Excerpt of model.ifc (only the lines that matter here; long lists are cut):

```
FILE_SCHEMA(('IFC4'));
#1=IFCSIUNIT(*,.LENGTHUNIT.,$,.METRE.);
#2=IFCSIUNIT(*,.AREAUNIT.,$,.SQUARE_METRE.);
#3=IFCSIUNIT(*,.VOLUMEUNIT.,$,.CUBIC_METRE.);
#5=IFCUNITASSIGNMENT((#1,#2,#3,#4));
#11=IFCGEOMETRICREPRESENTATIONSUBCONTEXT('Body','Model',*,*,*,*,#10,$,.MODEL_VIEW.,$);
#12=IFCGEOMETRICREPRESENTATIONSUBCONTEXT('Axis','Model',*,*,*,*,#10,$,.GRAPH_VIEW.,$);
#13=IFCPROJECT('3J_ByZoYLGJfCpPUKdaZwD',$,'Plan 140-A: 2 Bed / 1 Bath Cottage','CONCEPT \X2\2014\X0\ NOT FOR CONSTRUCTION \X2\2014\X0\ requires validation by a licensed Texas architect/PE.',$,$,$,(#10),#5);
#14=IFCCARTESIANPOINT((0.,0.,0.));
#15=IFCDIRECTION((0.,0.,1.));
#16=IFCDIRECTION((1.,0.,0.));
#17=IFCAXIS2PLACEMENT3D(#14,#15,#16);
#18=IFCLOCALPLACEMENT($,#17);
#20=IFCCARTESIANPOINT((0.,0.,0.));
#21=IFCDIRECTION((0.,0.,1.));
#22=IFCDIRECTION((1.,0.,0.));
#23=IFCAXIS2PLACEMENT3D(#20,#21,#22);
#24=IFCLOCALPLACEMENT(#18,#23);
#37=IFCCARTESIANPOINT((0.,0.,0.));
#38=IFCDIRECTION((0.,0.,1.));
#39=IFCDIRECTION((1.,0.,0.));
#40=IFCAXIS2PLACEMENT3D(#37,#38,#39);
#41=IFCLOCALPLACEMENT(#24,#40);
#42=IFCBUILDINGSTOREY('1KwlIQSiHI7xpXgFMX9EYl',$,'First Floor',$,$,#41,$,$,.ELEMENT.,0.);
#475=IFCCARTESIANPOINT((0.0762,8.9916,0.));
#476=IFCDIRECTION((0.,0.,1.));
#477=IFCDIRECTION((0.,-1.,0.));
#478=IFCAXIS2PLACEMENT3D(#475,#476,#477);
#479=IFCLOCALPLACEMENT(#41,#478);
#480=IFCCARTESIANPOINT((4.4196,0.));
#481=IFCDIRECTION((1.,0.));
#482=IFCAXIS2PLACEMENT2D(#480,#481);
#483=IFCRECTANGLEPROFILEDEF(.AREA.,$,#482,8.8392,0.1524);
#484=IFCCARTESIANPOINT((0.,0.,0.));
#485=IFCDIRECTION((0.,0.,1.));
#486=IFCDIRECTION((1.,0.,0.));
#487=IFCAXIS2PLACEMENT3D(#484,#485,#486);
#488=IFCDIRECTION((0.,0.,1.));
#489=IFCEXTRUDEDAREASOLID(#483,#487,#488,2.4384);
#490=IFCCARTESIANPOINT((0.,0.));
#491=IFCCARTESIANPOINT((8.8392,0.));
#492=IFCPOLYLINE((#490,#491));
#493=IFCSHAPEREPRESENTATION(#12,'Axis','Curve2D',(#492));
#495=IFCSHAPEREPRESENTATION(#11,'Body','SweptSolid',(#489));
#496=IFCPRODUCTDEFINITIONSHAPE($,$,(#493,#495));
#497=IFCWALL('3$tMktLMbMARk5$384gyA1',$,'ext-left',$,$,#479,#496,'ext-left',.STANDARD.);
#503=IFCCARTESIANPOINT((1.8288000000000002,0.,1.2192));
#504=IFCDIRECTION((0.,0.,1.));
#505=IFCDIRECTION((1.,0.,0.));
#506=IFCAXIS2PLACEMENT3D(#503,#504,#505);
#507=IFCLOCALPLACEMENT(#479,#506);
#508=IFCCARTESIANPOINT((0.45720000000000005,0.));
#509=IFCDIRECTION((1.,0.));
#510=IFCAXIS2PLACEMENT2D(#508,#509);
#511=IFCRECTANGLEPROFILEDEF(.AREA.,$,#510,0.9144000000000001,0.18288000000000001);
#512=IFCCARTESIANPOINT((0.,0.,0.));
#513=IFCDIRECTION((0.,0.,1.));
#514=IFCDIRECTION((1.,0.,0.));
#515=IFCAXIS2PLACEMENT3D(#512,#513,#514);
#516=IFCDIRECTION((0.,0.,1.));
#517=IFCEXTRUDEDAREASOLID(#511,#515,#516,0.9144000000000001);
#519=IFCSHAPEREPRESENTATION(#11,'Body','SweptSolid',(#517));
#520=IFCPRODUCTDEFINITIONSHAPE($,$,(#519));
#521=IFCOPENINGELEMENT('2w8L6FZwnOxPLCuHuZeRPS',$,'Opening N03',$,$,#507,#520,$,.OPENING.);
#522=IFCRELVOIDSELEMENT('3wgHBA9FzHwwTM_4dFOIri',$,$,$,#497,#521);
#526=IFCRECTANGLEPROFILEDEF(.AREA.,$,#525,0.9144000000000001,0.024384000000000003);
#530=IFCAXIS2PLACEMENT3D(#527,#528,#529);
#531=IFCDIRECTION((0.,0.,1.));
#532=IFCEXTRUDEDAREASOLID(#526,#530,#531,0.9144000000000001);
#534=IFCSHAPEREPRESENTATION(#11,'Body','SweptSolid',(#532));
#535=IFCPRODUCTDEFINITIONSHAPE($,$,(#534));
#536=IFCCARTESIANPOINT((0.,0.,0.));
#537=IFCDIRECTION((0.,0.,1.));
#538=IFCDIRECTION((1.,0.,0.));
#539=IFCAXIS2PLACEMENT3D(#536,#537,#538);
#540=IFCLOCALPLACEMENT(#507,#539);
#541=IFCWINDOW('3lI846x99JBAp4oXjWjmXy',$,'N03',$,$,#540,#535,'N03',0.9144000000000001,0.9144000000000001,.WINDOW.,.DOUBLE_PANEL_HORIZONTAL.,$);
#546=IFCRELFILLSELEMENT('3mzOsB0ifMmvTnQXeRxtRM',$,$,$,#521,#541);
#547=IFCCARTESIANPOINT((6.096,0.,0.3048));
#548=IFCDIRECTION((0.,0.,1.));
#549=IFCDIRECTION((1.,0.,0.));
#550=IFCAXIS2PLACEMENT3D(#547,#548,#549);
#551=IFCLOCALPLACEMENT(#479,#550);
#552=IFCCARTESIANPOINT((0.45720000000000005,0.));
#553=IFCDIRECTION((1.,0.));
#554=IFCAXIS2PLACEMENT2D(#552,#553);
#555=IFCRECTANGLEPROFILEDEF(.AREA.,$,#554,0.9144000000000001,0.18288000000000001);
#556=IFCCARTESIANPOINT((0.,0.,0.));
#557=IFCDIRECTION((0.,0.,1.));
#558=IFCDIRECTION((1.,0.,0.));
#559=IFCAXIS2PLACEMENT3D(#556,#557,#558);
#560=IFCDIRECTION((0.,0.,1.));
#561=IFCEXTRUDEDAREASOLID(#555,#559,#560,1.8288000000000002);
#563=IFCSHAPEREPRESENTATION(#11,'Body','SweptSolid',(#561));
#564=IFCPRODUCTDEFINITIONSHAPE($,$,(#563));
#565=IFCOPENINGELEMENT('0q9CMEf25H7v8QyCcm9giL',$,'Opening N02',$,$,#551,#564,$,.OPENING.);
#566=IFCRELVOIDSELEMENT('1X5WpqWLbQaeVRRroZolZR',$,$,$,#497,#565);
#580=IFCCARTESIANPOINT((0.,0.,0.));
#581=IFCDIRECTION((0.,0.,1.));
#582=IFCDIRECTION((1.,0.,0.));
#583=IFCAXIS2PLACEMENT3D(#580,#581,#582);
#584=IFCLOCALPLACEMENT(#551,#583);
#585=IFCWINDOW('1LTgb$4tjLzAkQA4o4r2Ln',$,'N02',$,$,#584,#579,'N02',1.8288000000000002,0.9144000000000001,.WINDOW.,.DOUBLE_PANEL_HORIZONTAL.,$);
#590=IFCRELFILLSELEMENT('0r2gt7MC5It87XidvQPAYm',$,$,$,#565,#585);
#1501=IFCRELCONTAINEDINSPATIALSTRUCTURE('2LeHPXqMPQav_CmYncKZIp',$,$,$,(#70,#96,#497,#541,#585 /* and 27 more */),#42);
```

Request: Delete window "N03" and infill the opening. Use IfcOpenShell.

```python
import ifcopenshell
import ifcopenshell.api.feature
import ifcopenshell.api.root
import ifcopenshell.geom
import ifcopenshell.util.shape

model = ifcopenshell.open("model.ifc")
settings = ifcopenshell.geom.settings()


def volume(element):
    """Net volume in cubic metres, openings subtracted."""
    shape = ifcopenshell.geom.create_shape(settings, element)
    return ifcopenshell.util.shape.get_volume(shape.geometry)


window = model.by_guid("3lI846x99JBAp4oXjWjmXy")
opening = window.FillsVoids[0].RelatingOpeningElement
wall = opening.VoidsElements[0].RelatingBuildingElement
before = volume(wall)

ifcopenshell.api.root.remove_product(model, product=window)
ifcopenshell.api.feature.remove_feature(model, feature=opening)

after = volume(wall)

print(f"wall volume {before:.3f} -> {after:.3f} m3")

model.write("model-out.ifc")
```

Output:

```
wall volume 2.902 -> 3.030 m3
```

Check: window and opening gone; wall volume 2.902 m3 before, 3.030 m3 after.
